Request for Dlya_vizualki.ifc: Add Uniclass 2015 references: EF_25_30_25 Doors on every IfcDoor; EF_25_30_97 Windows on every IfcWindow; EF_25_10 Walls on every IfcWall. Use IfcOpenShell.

First a look at what the model holds.

```python
import ifcopenshell

model = ifcopenshell.open("Dlya_vizualki.ifc")
print(model.schema)
print("classifications:", [c.Name for c in model.by_type("IfcClassification")])
for ifc_class in ("IfcDoor", "IfcRoof", "IfcStair", "IfcWall", "IfcWindow"):
    print(ifc_class, len(model.by_type(ifc_class)))
```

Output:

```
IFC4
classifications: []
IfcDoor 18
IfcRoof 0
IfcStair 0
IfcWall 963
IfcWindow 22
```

```python
import ifcopenshell
import ifcopenshell.api.classification

model = ifcopenshell.open("Dlya_vizualki.ifc")

system = ifcopenshell.api.classification.add_classification(model, classification="Uniclass 2015")

codes = {
    "IfcDoor": ("EF_25_30_25", "Doors"),
    "IfcWindow": ("EF_25_30_97", "Windows"),
    "IfcWall": ("EF_25_10", "Walls"),
}
for ifc_class, (code, name) in codes.items():
    products = model.by_type(ifc_class)
    ifcopenshell.api.classification.add_reference(
        model, products=products, classification=system, identification=code, name=name
    )
    print(code, len(products))

model.write("Dlya_vizualki_updated.ifc")
```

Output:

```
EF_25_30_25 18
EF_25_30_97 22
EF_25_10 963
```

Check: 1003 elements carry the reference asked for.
